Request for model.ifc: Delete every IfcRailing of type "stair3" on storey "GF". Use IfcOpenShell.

First a look at what the model holds.

```python
import ifcopenshell
import ifcopenshell.util.element

model = ifcopenshell.open("model.ifc")
print(model.schema)
storey = next(s for s in model.by_type("IfcBuildingStorey") if s.Name == "GF")
railings = [e for e in ifcopenshell.util.element.get_decomposition(storey) if e.is_a("IfcRailing")]
seen = {}
for e in railings:
    element_type = ifcopenshell.util.element.get_type(e)
    name = element_type.Name if element_type not in (None, e) else None
    seen[name] = seen.get(name, 0) + 1
for name, count in sorted(seen.items(), key=str):
    print(count, "x", name)
```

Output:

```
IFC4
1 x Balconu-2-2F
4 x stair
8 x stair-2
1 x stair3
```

```python
import ifcopenshell
import ifcopenshell.api.root
import ifcopenshell.util.element

model = ifcopenshell.open("model.ifc")

storey = next(s for s in model.by_type("IfcBuildingStorey") if s.Name == "GF")
railings = [e for e in ifcopenshell.util.element.get_decomposition(storey) if e.is_a("IfcRailing")]
targets = [e for e in railings if (t := ifcopenshell.util.element.get_type(e)) not in (None, e) and t.Name == "stair3"]

for e in targets:
    ifcopenshell.api.root.remove_product(model, product=e)
print(len(targets), "removed")

model.write("model-out.ifc")
```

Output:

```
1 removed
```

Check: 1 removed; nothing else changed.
